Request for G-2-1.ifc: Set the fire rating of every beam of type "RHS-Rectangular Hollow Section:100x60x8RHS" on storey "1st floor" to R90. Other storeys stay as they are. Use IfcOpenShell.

First a look at what the model holds.

```python
import ifcopenshell
import ifcopenshell.util.element

model = ifcopenshell.open("G-2-1.ifc")
print(model.schema)
storey = next(s for s in model.by_type("IfcBuildingStorey") if s.Name == "1st floor")
beams = [e for e in ifcopenshell.util.element.get_decomposition(storey) if e.is_a("IfcBeam")]
seen = {}
for e in beams:
    element_type = ifcopenshell.util.element.get_type(e)
    key = (element_type.Name if element_type != e and element_type else None, ifcopenshell.util.element.get_pset(e, "Pset_BeamCommon", "FireRating"))
    seen[key] = seen.get(key, 0) + 1
for (name, value), count in sorted(seen.items(), key=str):
    print(count, "x", name, "|", value)
```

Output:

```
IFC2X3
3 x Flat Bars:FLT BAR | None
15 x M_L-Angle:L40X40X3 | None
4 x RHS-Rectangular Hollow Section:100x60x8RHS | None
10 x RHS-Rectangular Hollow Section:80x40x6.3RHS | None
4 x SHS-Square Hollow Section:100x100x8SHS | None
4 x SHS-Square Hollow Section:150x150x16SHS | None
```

```python
import ifcopenshell
import ifcopenshell.api.pset
import ifcopenshell.util.element

model = ifcopenshell.open("G-2-1.ifc")

storey = next(s for s in model.by_type("IfcBuildingStorey") if s.Name == "1st floor")
beams = [e for e in ifcopenshell.util.element.get_decomposition(storey) if e.is_a("IfcBeam")]

count = 0
for e in beams:
    element_type = ifcopenshell.util.element.get_type(e)
    if element_type in (None, e) or element_type.Name != "RHS-Rectangular Hollow Section:100x60x8RHS":
        continue
    # add_pset returns the element's existing set when there is one.
    pset = ifcopenshell.api.pset.add_pset(model, product=e, name="Pset_BeamCommon")
    ifcopenshell.api.pset.edit_pset(model, pset=pset, properties={"FireRating": "R90"})
    count += 1

print(count, "beams updated")

model.write("G-2-1_updated.ifc")
```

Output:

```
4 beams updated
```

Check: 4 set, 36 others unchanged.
